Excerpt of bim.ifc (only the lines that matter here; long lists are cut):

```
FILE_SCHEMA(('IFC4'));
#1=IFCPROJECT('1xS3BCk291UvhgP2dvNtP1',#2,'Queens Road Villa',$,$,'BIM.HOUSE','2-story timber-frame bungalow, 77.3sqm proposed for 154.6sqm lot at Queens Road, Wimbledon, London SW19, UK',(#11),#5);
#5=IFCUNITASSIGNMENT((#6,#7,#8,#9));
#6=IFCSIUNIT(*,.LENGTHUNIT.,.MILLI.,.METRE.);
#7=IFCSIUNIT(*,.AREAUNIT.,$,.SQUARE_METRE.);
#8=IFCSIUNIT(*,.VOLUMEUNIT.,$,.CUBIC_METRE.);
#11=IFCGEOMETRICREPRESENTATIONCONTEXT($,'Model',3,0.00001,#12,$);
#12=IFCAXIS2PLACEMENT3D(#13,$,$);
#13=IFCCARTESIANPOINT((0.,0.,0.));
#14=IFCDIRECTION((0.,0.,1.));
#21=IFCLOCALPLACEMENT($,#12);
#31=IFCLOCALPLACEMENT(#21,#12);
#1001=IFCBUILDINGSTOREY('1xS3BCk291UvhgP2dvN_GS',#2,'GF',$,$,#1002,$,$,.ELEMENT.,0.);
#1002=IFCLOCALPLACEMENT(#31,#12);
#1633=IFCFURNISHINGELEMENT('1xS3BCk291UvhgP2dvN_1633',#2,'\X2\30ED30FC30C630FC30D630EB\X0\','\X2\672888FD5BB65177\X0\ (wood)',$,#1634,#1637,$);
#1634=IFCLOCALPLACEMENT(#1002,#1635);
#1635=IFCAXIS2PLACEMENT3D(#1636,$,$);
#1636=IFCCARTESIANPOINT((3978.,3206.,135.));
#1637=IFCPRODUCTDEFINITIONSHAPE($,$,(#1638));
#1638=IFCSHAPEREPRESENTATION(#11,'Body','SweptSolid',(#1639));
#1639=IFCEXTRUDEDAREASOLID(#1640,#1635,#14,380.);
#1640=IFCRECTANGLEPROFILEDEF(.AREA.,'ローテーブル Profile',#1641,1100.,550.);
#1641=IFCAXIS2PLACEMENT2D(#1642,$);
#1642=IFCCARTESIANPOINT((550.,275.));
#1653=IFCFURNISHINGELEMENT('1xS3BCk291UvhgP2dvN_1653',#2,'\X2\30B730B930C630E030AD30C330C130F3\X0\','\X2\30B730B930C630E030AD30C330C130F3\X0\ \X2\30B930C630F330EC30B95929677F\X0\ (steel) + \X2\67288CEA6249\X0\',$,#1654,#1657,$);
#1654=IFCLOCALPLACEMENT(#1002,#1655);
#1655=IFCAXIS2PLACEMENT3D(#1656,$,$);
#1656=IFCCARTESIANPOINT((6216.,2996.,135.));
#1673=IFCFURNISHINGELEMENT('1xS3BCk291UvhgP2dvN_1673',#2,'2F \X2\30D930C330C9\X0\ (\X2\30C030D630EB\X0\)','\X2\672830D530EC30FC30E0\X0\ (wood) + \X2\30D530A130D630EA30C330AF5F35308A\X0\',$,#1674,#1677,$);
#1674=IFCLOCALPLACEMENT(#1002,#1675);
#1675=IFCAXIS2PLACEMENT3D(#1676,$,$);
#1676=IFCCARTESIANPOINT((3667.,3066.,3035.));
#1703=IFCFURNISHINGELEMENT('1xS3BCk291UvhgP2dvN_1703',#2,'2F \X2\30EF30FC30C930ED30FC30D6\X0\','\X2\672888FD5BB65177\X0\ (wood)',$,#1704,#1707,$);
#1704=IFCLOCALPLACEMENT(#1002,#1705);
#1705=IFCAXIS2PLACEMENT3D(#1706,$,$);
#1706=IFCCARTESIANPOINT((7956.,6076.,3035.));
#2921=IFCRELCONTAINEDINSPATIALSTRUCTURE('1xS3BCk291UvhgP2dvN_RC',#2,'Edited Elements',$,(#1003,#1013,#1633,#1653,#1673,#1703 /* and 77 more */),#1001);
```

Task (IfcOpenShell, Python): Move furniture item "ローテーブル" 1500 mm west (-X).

```python
import ifcopenshell
import ifcopenshell.api.geometry
import ifcopenshell.util.placement
import ifcopenshell.util.unit

model = ifcopenshell.open("bim.ifc")
unit_scale = ifcopenshell.util.unit.calculate_unit_scale(model)

item = model.by_guid("1xS3BCk291UvhgP2dvN_1633")
matrix = ifcopenshell.util.placement.get_local_placement(item.ObjectPlacement)
matrix[0, 3] -= 1.5 / unit_scale
ifcopenshell.api.geometry.edit_object_placement(model, product=item, matrix=matrix, is_si=False)

print(ifcopenshell.util.placement.get_local_placement(item.ObjectPlacement).round(3) + 0.0)

model.write("bim_rev.ifc")
```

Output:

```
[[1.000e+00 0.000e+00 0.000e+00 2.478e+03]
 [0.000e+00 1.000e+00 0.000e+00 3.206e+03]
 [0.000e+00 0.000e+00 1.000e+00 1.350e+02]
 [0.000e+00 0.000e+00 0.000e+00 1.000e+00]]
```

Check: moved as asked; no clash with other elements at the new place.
